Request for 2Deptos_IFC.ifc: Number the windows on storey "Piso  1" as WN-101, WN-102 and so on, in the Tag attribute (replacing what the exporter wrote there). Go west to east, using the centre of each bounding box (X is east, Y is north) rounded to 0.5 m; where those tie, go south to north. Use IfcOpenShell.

First a look at what the model holds.

```python
import ifcopenshell
import ifcopenshell.util.element
import ifcopenshell.util.placement

model = ifcopenshell.open("2Deptos_IFC.ifc")
print(model.schema)
storey = next(s for s in model.by_type("IfcBuildingStorey") if s.Name == "Piso  1")
windows = [e for e in ifcopenshell.util.element.get_decomposition(storey) if e.is_a("IfcWindow")]
for e in sorted(windows, key=lambda e: e.id()):
    origin = ifcopenshell.util.placement.get_local_placement(e.ObjectPlacement)[:3, 3]
    print(e.id(), e.Tag, e.Name, origin.round(2) + 0.0, sep=" | ")
```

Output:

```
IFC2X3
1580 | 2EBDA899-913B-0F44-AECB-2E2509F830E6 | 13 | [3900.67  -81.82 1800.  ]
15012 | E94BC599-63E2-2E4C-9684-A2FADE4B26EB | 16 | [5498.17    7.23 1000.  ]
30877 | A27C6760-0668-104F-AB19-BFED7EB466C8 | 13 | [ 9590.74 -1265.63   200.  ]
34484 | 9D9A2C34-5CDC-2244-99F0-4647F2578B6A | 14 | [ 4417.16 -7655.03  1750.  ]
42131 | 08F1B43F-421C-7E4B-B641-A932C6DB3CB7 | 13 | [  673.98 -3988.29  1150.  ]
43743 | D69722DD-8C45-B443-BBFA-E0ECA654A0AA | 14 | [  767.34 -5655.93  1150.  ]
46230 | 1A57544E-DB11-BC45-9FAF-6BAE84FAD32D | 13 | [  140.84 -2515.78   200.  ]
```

```python
import ifcopenshell
import ifcopenshell.geom
import ifcopenshell.util.element
import ifcopenshell.util.shape

model = ifcopenshell.open("2Deptos_IFC.ifc")
settings = ifcopenshell.geom.settings()
settings.set("use-world-coords", True)


def centre(element):
    shape = ifcopenshell.geom.create_shape(settings, element)
    return ifcopenshell.util.shape.get_bbox_centroid(shape.geometry)


storey = next(s for s in model.by_type("IfcBuildingStorey") if s.Name == "Piso  1")
windows = [e for e in ifcopenshell.util.element.get_decomposition(storey) if e.is_a("IfcWindow")]

# Insertion points can sit at a corner or the storey origin, so sort by the geometry (in metres).
centres = {e: centre(e) for e in windows}
windows.sort(key=lambda e: (round(centres[e][0] / 0.5), centres[e][1]))

for i, e in enumerate(windows, start=1):
    number = f"WN-1{i:02d}"
    e.Tag = number
    print(e.id(), number)

model.write("2Deptos_IFC_rev.ifc")
```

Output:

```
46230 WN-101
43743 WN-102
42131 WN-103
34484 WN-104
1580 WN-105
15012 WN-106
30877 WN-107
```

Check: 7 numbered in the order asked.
